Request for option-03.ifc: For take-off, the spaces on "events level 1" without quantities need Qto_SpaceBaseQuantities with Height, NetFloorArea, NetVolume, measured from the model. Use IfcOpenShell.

First a look at what the model holds.

```python
import ifcopenshell
import ifcopenshell.util.element
import ifcopenshell.util.unit

model = ifcopenshell.open("option-03.ifc")
print(model.schema)
for unit_type in ("LENGTHUNIT", "AREAUNIT", "VOLUMEUNIT"):
    print(unit_type, ifcopenshell.util.unit.calculate_unit_scale(model, unit_type))
storey = next(s for s in model.by_type("IfcBuildingStorey") if s.Name == "events level 1")
spaces = [e for e in ifcopenshell.util.element.get_decomposition(storey) if e.is_a("IfcSpace")]
for e in sorted(spaces, key=lambda e: e.id()):
    print(e.id(), e.is_a(), e.Name, list(ifcopenshell.util.element.get_psets(e, qtos_only=True)), sep=" | ")
```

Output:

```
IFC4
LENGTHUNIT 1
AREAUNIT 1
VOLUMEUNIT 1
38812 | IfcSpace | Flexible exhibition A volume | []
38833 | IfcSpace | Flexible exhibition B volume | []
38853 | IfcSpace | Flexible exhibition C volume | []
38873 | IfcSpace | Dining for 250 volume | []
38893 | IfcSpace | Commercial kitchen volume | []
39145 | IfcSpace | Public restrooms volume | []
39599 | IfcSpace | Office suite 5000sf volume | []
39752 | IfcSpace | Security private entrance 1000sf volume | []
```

```python
import ifcopenshell
import ifcopenshell.api.pset
import ifcopenshell.geom
import ifcopenshell.util.element
import ifcopenshell.util.shape
import ifcopenshell.util.unit

model = ifcopenshell.open("option-03.ifc")
unit_scale = ifcopenshell.util.unit.calculate_unit_scale(model)
area_scale = ifcopenshell.util.unit.calculate_unit_scale(model, "AREAUNIT")
volume_scale = ifcopenshell.util.unit.calculate_unit_scale(model, "VOLUMEUNIT")
settings = ifcopenshell.geom.settings()

storey = next(s for s in model.by_type("IfcBuildingStorey") if s.Name == "events level 1")
spaces = [e for e in ifcopenshell.util.element.get_decomposition(storey) if e.is_a("IfcSpace")]

for e in sorted(spaces, key=lambda e: e.id()):
    if ifcopenshell.util.element.get_psets(e, qtos_only=True, should_inherit=False):
        continue
    # Geometry comes back in metres, in the element's own axes.
    shape = ifcopenshell.geom.create_shape(settings, e)
    values = {
        "Height": ifcopenshell.util.shape.get_z(shape.geometry) / unit_scale,
        "NetFloorArea": ifcopenshell.util.shape.get_footprint_area(shape.geometry) / area_scale,
        "NetVolume": ifcopenshell.util.shape.get_volume(shape.geometry) / volume_scale,
    }
    qto = ifcopenshell.api.pset.add_qto(model, product=e, name="Qto_SpaceBaseQuantities")
    ifcopenshell.api.pset.edit_qto(model, qto=qto, properties=values)
    print(e.id(), {k: round(v, 3) for k, v in values.items()})

model.write("option-03_v2.ifc")
```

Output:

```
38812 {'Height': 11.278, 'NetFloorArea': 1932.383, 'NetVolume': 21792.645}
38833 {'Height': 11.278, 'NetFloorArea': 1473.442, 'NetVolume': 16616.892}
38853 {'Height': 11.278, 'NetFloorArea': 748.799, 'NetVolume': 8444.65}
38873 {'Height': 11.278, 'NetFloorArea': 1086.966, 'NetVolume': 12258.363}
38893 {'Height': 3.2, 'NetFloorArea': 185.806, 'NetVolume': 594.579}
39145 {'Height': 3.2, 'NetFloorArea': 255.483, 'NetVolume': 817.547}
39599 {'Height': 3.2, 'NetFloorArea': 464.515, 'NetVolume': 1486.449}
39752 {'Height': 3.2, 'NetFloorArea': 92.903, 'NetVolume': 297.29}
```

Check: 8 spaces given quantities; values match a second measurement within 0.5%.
